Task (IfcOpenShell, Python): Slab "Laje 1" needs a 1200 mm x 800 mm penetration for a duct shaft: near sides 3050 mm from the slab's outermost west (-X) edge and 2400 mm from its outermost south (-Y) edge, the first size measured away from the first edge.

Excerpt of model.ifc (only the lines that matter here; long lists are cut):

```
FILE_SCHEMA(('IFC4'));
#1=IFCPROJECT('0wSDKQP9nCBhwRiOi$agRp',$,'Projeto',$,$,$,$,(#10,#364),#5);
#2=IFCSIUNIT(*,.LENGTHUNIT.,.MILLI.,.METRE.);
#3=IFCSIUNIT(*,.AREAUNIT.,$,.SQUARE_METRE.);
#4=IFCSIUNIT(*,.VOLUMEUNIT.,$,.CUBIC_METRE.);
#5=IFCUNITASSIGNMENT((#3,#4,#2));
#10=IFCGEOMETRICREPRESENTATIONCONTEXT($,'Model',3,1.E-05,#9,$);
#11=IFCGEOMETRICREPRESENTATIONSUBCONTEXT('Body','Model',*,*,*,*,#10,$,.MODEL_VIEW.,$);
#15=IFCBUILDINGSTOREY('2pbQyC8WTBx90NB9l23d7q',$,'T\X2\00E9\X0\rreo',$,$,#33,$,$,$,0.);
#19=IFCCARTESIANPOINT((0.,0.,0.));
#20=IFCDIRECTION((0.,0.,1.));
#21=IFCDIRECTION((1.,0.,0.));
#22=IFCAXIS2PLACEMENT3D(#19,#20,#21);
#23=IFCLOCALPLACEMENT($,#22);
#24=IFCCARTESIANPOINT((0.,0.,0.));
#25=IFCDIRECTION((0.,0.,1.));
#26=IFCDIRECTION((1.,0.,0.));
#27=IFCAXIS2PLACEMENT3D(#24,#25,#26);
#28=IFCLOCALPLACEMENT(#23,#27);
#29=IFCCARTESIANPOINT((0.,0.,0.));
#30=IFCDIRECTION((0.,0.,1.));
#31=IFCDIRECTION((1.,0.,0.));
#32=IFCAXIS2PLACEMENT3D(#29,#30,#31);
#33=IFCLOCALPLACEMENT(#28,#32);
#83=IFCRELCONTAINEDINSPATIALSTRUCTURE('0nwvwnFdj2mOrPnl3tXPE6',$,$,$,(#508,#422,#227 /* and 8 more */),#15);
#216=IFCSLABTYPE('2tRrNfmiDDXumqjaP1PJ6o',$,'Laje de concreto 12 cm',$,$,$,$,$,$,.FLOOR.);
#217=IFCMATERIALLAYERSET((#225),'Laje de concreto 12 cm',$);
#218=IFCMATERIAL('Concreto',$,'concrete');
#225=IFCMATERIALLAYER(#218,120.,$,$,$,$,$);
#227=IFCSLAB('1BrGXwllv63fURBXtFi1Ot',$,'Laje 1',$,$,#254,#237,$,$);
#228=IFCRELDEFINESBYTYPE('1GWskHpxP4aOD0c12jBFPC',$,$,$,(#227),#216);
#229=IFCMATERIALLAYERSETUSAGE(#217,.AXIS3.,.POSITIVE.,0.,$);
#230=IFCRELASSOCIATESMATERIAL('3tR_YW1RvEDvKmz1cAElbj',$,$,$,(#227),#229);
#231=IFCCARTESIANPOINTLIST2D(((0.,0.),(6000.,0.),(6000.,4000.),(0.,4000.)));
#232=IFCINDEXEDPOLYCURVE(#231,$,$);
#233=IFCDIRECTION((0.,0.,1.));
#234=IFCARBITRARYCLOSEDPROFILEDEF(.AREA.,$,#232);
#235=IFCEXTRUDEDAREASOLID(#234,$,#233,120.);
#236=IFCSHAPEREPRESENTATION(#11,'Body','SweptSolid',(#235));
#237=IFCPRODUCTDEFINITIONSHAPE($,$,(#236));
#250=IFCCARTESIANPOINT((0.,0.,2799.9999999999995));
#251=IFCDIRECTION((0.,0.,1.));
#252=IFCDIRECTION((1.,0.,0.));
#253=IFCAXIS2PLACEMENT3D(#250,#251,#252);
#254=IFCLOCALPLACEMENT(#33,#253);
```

```python
import numpy as np
import ifcopenshell
import ifcopenshell.api.feature
import ifcopenshell.api.geometry
import ifcopenshell.api.root
import ifcopenshell.geom
import ifcopenshell.util.placement
import ifcopenshell.util.representation
import ifcopenshell.util.shape
import ifcopenshell.util.unit

model = ifcopenshell.open("model.ifc")
unit_scale = ifcopenshell.util.unit.calculate_unit_scale(model)
settings = ifcopenshell.geom.settings()


def volume(element):
    """Net volume in cubic metres, openings subtracted."""
    shape = ifcopenshell.geom.create_shape(settings, element)
    return ifcopenshell.util.shape.get_volume(shape.geometry)


slab = model.by_guid("1BrGXwllv63fURBXtFi1Ot")
before = volume(slab)

# Extent in the slab's own axes, in metres. The edges named are its -X and -Y sides.
slab_shape = ifcopenshell.geom.create_shape(settings, slab)
vertices = ifcopenshell.util.shape.get_vertices(slab_shape.geometry)
x_min, y_min, bottom = vertices.min(axis=0)
top = vertices[:, 2].max()

opening = ifcopenshell.api.root.create_entity(model, ifc_class="IfcOpeningElement", name="Duct shaft opening", predefined_type="OPENING")
context = ifcopenshell.util.representation.get_context(model, "Model", "Body", "MODEL_VIEW")
width, depth = 1.2, 0.8
outline = [(0.0, 0.0), (width, 0.0), (width, depth), (0.0, depth), (0.0, 0.0)]
# Overshoot both faces by 50 mm so the cut is clean.
shape = ifcopenshell.api.geometry.add_slab_representation(
    model, context=context, depth=top - bottom + 0.1, polyline=outline
)
ifcopenshell.api.geometry.assign_representation(model, product=opening, representation=shape)

matrix = ifcopenshell.util.placement.get_local_placement(slab.ObjectPlacement)
matrix[:, 3] = matrix @ np.append(np.array([x_min + 3.05, y_min + 2.4, bottom - 0.05]) / unit_scale, 1.0)
ifcopenshell.api.geometry.edit_object_placement(model, product=opening, matrix=matrix, is_si=False)
ifcopenshell.api.feature.add_feature(model, feature=opening, element=slab)

after = volume(slab)

print(f"slab volume {before:.3f} -> {after:.3f} m3")

model.write("model_updated.ifc")
```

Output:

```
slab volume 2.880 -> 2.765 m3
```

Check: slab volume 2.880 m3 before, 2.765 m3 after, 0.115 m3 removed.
